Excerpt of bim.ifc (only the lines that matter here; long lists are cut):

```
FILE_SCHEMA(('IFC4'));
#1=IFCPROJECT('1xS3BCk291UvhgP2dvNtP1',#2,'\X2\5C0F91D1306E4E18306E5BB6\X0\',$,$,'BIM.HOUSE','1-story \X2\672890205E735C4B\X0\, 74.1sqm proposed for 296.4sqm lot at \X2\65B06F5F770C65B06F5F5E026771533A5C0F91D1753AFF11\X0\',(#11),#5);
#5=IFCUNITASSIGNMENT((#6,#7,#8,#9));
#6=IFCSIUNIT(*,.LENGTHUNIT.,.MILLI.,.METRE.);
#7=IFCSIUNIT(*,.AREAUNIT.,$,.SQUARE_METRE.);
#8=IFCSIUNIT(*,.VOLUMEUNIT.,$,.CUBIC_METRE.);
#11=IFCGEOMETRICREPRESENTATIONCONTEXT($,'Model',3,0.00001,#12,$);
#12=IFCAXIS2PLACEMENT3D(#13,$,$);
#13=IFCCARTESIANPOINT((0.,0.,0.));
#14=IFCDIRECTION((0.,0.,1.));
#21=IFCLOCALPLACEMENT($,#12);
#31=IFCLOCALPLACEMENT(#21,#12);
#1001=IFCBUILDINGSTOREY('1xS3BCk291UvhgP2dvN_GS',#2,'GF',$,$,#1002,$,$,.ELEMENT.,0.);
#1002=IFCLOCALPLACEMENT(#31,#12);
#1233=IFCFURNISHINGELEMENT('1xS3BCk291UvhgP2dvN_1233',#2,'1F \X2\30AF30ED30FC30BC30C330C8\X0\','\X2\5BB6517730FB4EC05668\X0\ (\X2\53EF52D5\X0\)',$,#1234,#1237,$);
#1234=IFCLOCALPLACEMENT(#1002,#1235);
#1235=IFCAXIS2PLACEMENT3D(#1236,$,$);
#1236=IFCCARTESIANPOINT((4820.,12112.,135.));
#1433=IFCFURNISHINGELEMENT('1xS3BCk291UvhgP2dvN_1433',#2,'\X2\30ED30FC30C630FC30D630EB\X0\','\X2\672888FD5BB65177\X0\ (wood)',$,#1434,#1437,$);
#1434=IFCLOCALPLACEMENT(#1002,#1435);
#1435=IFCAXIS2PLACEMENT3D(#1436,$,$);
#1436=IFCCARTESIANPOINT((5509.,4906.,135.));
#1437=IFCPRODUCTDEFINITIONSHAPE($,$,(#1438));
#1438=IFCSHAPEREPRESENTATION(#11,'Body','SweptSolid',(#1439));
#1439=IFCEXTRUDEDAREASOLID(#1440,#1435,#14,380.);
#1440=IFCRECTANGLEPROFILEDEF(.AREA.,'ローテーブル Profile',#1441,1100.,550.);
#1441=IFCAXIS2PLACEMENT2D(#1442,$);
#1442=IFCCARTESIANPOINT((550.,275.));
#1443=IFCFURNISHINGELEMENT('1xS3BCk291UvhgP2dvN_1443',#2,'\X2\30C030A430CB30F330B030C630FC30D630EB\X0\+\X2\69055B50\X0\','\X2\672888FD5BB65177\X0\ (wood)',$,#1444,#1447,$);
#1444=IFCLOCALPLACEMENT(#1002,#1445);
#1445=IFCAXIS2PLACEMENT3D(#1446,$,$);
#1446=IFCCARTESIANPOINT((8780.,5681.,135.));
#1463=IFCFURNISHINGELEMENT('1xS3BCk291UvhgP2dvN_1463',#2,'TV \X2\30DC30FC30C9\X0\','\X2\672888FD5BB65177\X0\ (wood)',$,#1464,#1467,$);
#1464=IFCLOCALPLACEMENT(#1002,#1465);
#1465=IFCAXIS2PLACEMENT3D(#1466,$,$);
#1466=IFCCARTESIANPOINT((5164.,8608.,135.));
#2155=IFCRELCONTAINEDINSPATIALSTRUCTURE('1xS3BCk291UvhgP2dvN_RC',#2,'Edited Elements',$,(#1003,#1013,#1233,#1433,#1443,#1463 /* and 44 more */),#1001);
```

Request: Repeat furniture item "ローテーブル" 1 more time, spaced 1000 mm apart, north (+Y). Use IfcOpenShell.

```python
import numpy as np
import ifcopenshell
import ifcopenshell.api.geometry
import ifcopenshell.api.root
import ifcopenshell.util.element
import ifcopenshell.util.placement
import ifcopenshell.util.unit

model = ifcopenshell.open("bim.ifc")
unit_scale = ifcopenshell.util.unit.calculate_unit_scale(model)


def reuse_history(source, copy):
    """copy_class also copies each property set's owner history, people and application; keep the originals."""
    for rel in copy.IsDefinedBy:
        if rel.is_a("IfcRelDefinesByProperties") and (history := rel.RelatingPropertyDefinition.OwnerHistory):
            rel.RelatingPropertyDefinition.OwnerHistory = source.OwnerHistory
            ifcopenshell.util.element.remove_deep2(model, history)


source = model.by_id(1433)
base = ifcopenshell.util.placement.get_local_placement(source.ObjectPlacement)
step = np.array([0.0, 1.0, 0.0]) * 1 / unit_scale

for i in range(1, 2):
    copy = ifcopenshell.api.root.copy_class(model, product=source)
    copy.Representation = ifcopenshell.util.element.copy_deep(
        model, source.Representation, exclude=["IfcGeometricRepresentationContext", "IfcRepresentationMap"]
    )
    reuse_history(source, copy)
    matrix = base.copy()
    matrix[:3, 3] += i * step
    print("added at", matrix[:3, 3].round(3) + 0.0)
    ifcopenshell.api.geometry.edit_object_placement(model, product=copy, matrix=matrix, is_si=False)

model.write("bim_rev.ifc")
```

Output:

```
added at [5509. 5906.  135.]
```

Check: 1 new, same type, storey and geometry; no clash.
